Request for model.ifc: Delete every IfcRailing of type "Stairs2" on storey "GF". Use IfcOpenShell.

First a look at what the model holds.

```python
import ifcopenshell
import ifcopenshell.util.element

model = ifcopenshell.open("model.ifc")
print(model.schema)
storey = next(s for s in model.by_type("IfcBuildingStorey") if s.Name == "GF")
railings = [e for e in ifcopenshell.util.element.get_decomposition(storey) if e.is_a("IfcRailing")]
seen = {}
for e in railings:
    element_type = ifcopenshell.util.element.get_type(e)
    name = element_type.Name if element_type not in (None, e) else None
    seen[name] = seen.get(name, 0) + 1
for name, count in sorted(seen.items(), key=str):
    print(count, "x", name)
```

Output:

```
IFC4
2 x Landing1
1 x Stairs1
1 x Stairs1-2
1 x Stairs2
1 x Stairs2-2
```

```python
import ifcopenshell
import ifcopenshell.api.root
import ifcopenshell.util.element

model = ifcopenshell.open("model.ifc")

storey = next(s for s in model.by_type("IfcBuildingStorey") if s.Name == "GF")
railings = [e for e in ifcopenshell.util.element.get_decomposition(storey) if e.is_a("IfcRailing")]
targets = [e for e in railings if (t := ifcopenshell.util.element.get_type(e)) not in (None, e) and t.Name == "Stairs2"]

for e in targets:
    ifcopenshell.api.root.remove_product(model, product=e)
print(len(targets), "removed")

model.write("model_edited.ifc")
```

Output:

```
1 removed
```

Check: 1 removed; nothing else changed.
